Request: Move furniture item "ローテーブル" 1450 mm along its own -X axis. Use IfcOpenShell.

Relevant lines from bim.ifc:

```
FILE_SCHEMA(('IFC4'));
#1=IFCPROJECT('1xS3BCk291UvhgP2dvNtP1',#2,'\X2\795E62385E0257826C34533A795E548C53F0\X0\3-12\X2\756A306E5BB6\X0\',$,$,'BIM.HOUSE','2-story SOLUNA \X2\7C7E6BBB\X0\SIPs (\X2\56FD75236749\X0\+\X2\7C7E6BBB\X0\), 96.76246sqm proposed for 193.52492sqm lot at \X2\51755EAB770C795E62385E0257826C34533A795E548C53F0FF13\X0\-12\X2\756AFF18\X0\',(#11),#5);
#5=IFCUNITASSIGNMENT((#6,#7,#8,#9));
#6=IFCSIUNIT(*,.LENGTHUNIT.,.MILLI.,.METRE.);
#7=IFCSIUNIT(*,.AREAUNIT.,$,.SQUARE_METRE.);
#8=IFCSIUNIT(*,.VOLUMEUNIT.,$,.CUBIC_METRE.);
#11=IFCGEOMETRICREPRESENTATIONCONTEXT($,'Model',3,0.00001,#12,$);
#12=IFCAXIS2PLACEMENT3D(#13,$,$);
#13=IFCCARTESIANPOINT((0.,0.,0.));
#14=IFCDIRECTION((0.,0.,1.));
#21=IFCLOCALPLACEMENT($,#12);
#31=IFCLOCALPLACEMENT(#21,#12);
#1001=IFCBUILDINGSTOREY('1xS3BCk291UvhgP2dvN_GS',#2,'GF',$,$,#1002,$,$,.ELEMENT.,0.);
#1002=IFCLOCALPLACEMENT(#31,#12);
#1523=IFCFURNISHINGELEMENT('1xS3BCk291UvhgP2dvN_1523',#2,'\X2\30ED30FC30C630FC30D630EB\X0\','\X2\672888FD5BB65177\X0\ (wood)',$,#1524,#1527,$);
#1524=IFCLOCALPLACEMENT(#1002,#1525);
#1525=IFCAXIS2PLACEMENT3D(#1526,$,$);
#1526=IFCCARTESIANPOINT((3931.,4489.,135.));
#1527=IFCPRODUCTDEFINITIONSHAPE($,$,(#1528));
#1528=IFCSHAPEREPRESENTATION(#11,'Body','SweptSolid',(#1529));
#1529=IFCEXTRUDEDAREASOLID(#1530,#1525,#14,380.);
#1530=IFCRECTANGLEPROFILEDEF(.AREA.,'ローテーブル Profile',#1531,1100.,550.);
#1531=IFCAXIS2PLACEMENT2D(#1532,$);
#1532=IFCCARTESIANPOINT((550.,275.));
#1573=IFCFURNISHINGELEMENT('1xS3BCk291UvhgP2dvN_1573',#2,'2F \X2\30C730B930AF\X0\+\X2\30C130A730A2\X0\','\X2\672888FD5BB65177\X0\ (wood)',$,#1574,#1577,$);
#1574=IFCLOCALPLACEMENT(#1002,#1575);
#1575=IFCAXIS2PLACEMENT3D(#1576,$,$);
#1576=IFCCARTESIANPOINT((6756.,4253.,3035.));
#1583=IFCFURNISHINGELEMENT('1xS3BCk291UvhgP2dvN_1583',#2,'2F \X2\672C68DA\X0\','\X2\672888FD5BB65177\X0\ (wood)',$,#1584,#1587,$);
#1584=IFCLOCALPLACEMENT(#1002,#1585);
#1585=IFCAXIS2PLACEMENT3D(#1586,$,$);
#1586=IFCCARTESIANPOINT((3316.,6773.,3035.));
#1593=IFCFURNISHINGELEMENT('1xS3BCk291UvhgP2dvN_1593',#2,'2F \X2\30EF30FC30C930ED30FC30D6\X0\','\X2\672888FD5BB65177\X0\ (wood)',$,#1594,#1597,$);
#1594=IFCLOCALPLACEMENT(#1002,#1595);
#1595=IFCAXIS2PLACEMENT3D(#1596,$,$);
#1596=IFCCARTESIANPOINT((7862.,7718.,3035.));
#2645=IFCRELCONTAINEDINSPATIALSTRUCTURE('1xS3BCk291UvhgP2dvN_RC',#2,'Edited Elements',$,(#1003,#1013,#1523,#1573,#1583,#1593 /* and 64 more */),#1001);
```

```python
import ifcopenshell
import ifcopenshell.api.geometry
import ifcopenshell.util.placement
import ifcopenshell.util.unit

model = ifcopenshell.open("bim.ifc")
unit_scale = ifcopenshell.util.unit.calculate_unit_scale(model)

item = model.by_id(1523)
matrix = ifcopenshell.util.placement.get_local_placement(item.ObjectPlacement)
matrix[:3, 3] -= matrix[:3, 0] * 1.45 / unit_scale
ifcopenshell.api.geometry.edit_object_placement(model, product=item, matrix=matrix, is_si=False)

print(ifcopenshell.util.placement.get_local_placement(item.ObjectPlacement).round(3) + 0.0)

model.write("bim_updated.ifc")
```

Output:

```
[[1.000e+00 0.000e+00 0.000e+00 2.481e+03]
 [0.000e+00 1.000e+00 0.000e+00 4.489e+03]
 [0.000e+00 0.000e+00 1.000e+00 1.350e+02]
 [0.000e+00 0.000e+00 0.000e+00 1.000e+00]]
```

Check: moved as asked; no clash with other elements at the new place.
